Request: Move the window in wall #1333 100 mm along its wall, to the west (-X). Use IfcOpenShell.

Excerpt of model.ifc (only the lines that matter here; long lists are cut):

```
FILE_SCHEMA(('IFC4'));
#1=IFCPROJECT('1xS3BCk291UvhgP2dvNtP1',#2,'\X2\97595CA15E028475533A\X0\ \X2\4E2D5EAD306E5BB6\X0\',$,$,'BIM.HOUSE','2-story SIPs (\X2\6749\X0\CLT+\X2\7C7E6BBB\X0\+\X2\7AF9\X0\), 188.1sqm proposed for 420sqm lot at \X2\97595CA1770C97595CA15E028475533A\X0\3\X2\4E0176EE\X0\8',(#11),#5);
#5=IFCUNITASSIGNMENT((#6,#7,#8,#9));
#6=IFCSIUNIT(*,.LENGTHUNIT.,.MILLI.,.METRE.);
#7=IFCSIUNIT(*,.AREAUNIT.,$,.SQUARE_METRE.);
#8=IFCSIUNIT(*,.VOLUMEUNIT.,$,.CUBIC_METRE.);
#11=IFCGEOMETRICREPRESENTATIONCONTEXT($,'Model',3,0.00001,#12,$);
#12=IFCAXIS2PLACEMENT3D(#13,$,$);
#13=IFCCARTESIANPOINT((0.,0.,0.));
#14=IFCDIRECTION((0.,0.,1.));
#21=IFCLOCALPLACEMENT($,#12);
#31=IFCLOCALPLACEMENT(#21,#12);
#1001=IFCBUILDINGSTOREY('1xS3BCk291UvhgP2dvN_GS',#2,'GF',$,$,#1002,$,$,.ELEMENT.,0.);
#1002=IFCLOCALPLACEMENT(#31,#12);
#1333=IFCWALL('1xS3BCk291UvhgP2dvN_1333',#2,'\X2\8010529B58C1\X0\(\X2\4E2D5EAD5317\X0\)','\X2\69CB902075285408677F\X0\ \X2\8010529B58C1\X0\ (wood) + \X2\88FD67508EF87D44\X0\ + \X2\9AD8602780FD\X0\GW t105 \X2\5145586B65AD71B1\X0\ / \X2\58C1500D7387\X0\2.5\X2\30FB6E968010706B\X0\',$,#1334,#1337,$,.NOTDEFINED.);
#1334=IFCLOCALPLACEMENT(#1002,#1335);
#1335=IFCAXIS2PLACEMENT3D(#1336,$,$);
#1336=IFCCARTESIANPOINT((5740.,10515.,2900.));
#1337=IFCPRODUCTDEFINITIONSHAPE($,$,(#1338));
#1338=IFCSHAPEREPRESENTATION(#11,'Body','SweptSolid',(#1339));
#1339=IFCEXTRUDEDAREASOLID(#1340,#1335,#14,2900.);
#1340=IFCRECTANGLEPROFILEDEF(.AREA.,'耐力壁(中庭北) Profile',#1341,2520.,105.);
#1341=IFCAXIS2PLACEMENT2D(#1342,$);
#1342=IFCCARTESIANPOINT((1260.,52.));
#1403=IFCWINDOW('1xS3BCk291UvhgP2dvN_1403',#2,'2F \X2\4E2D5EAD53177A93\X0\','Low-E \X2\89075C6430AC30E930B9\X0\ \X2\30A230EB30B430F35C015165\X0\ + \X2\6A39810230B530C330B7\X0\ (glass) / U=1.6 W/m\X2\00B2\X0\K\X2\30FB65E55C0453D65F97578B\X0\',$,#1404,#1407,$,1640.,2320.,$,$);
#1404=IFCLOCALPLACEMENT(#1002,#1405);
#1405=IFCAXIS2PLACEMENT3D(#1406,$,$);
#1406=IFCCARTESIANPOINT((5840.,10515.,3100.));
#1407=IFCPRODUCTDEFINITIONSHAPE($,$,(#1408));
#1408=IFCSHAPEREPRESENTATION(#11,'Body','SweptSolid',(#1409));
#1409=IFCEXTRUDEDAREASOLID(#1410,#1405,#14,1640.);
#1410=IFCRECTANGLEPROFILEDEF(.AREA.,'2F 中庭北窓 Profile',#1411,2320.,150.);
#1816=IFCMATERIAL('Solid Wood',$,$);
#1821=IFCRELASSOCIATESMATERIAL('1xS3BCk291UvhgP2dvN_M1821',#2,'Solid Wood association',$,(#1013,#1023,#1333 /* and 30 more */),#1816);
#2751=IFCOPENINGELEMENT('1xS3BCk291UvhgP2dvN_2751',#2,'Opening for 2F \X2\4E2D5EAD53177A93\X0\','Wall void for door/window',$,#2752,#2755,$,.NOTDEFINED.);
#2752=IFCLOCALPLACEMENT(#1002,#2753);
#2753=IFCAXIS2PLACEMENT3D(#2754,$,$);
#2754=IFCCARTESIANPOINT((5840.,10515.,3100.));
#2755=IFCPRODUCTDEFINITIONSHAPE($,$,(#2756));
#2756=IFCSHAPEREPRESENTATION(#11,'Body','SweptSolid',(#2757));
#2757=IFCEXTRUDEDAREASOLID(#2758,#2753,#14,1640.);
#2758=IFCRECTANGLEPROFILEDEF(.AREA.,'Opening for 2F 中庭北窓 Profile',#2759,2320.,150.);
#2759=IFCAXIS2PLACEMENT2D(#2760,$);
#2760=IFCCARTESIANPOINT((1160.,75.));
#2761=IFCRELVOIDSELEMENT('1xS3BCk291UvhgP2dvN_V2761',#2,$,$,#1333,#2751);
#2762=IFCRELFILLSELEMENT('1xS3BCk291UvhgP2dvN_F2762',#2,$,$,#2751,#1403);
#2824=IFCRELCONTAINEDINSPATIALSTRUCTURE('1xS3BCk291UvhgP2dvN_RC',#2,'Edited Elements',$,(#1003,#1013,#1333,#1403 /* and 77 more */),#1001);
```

```python
import ifcopenshell
import ifcopenshell.api.geometry
import ifcopenshell.util.placement
import ifcopenshell.util.unit

model = ifcopenshell.open("model.ifc")
unit_scale = ifcopenshell.util.unit.calculate_unit_scale(model)

window = model.by_guid("1xS3BCk291UvhgP2dvN_1403")
opening = window.FillsVoids[0].RelatingOpeningElement
wall = opening.VoidsElements[0].RelatingBuildingElement

wall_matrix = ifcopenshell.util.placement.get_local_placement(wall.ObjectPlacement)
shift = wall_matrix[:3, 0] * -0.1 / unit_scale
before = ifcopenshell.util.placement.get_local_placement(window.ObjectPlacement)[:3, 3].copy()

# The window is not placed relative to its opening, so move both.
for product in (opening, window):
    matrix = ifcopenshell.util.placement.get_local_placement(product.ObjectPlacement)
    matrix[:3, 3] += shift
    ifcopenshell.api.geometry.edit_object_placement(model, product=product, matrix=matrix, is_si=False)

after = ifcopenshell.util.placement.get_local_placement(window.ObjectPlacement)[:3, 3]
print("window moved by", (after - before).round(3) + 0.0)

model.write("model-out.ifc")
```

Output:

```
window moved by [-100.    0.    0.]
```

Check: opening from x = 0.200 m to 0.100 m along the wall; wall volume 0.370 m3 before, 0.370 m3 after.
